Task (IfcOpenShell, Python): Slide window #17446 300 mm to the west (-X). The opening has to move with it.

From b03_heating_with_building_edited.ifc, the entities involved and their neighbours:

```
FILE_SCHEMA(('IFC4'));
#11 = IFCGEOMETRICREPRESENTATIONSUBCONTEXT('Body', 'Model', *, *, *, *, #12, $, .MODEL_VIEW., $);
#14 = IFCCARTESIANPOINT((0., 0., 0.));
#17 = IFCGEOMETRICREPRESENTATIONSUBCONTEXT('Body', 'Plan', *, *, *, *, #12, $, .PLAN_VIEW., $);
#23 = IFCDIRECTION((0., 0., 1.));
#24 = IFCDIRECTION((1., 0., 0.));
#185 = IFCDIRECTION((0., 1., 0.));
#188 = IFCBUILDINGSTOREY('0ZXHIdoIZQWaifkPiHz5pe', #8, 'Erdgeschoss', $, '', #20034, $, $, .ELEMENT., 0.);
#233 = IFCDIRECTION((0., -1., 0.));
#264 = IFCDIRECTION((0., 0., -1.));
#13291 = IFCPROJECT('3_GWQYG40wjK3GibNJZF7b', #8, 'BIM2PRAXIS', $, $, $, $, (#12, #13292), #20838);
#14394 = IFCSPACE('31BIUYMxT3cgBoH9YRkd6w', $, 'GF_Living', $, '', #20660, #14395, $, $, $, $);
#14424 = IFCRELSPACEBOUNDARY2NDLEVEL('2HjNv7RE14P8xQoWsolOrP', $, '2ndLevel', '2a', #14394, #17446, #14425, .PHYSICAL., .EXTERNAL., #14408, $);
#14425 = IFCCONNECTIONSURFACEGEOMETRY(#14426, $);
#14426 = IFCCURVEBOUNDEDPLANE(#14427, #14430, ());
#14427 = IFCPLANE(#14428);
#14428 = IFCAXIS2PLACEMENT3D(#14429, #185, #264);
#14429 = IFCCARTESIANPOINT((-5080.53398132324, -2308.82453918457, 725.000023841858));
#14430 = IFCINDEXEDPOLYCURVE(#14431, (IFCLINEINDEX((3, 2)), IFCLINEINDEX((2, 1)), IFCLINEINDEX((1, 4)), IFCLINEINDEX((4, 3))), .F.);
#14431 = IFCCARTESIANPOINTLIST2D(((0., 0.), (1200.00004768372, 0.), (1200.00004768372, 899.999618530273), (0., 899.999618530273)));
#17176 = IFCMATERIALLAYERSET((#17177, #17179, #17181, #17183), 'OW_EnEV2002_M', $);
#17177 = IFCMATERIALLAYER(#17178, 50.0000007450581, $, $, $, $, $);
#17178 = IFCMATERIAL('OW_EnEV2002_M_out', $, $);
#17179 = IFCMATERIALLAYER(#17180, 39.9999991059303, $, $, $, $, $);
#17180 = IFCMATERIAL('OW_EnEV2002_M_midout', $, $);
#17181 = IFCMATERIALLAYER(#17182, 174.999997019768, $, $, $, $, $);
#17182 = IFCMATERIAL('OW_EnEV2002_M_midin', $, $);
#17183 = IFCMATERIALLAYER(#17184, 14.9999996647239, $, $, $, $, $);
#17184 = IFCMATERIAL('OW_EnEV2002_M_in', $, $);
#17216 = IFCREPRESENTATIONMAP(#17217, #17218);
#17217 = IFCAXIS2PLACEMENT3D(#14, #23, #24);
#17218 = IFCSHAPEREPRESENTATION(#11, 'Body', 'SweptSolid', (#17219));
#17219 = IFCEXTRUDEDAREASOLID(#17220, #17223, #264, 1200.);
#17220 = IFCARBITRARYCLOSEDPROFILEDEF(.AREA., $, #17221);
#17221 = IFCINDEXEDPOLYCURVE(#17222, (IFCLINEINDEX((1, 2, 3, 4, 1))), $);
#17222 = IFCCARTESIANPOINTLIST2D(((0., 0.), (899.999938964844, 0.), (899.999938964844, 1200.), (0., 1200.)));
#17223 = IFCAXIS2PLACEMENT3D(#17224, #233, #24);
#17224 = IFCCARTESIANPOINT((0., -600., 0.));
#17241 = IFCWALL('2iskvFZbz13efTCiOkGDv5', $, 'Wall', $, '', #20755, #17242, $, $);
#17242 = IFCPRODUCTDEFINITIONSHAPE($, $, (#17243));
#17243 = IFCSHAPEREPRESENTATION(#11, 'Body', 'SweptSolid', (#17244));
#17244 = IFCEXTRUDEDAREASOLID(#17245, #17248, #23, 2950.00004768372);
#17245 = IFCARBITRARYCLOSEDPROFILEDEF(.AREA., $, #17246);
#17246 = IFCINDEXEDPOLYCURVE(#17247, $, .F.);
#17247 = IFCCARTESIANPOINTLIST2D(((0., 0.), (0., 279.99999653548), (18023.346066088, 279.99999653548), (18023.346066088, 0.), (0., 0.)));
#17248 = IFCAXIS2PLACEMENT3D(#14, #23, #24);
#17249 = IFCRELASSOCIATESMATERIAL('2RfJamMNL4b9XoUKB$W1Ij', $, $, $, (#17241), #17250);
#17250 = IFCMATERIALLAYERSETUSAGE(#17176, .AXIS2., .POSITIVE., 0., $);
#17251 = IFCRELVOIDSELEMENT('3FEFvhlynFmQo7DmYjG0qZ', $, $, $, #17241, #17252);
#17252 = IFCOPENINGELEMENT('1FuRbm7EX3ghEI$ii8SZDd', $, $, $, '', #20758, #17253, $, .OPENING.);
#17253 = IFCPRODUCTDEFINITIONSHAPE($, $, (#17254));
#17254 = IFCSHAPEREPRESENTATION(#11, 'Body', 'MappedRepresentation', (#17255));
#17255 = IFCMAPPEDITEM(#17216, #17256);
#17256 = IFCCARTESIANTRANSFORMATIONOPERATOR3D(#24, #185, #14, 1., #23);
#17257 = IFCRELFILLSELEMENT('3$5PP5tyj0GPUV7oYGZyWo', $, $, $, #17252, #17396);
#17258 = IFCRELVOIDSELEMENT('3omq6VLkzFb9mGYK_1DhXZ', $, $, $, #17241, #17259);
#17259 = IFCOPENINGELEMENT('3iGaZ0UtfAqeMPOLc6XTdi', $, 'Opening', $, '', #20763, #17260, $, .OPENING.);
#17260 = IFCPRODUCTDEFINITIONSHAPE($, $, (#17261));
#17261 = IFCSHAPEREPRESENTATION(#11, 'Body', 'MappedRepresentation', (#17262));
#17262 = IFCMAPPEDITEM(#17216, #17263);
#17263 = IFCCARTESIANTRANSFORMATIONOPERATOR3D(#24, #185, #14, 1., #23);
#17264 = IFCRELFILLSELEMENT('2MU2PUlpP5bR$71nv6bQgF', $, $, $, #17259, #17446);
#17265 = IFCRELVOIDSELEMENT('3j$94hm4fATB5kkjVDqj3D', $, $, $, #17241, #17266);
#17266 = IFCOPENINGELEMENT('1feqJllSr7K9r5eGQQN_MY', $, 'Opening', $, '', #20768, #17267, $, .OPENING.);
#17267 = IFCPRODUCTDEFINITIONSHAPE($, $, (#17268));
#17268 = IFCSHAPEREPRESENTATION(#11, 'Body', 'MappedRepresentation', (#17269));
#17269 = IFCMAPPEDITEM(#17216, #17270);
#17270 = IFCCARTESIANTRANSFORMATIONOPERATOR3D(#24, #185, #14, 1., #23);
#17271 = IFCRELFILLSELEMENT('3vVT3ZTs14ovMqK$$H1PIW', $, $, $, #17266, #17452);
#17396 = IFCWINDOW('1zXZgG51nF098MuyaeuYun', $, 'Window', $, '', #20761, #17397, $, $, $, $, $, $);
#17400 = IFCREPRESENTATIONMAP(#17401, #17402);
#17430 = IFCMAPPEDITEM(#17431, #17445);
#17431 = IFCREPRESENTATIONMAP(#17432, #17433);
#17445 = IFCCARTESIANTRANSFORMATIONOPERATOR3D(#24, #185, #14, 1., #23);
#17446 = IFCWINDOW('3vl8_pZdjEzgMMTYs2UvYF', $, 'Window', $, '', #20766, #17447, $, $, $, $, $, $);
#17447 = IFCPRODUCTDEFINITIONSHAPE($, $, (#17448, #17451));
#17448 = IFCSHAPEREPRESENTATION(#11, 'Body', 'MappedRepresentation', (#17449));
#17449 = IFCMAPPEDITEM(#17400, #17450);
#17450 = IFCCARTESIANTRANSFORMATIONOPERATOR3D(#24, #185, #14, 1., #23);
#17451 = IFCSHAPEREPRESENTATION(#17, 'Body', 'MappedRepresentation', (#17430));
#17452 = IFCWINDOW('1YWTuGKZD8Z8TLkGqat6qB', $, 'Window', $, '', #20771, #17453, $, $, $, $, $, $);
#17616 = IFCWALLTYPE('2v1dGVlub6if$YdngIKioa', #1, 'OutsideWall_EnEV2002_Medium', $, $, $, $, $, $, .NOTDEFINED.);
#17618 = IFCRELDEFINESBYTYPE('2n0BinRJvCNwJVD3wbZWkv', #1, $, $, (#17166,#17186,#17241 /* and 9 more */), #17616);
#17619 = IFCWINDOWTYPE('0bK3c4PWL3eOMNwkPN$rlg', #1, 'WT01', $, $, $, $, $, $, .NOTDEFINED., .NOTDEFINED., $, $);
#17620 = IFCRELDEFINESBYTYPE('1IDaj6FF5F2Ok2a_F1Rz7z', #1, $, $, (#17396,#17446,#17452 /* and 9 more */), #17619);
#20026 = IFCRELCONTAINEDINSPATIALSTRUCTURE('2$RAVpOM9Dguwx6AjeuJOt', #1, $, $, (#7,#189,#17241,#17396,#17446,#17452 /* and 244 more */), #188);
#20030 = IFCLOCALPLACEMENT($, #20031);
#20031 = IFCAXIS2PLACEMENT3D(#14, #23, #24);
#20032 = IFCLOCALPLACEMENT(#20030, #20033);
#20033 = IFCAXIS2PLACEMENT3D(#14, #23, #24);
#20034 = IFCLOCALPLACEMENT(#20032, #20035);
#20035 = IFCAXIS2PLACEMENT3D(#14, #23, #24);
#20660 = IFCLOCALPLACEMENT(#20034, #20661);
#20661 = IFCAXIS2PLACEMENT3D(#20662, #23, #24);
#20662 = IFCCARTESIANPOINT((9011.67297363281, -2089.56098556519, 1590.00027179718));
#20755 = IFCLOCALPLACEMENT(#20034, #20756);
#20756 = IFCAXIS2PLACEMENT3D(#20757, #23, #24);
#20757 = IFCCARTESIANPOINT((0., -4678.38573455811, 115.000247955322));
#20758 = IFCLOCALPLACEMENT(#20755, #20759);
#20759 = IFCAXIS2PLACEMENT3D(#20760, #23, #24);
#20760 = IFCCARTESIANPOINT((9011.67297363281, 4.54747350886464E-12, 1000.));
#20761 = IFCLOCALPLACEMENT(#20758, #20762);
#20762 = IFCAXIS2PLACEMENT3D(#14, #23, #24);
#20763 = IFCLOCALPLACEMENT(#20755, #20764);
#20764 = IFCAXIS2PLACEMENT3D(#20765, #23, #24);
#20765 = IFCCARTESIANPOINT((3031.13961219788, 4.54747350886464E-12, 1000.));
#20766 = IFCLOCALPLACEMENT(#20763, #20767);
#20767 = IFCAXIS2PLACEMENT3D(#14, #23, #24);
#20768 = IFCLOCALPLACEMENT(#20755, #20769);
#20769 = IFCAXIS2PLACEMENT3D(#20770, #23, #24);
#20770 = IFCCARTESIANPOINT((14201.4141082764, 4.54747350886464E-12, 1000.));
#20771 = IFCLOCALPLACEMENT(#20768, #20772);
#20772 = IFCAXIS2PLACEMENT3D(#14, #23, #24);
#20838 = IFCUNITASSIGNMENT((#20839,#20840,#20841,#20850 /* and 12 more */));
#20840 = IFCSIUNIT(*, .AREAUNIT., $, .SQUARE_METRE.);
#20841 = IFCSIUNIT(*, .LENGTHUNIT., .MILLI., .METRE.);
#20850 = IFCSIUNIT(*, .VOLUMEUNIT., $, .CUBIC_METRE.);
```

```python
import numpy as np
import ifcopenshell
import ifcopenshell.api.geometry
import ifcopenshell.util.placement

model = ifcopenshell.open("b03_heating_with_building_edited.ifc")

window = model.by_guid("3vl8_pZdjEzgMMTYs2UvYF")
opening = window.FillsVoids[0].RelatingOpeningElement
wall = opening.VoidsElements[0].RelatingBuildingElement

wall_matrix = ifcopenshell.util.placement.get_local_placement(wall.ObjectPlacement)
shift = wall_matrix[:3, 0] * -300.0
before = ifcopenshell.util.placement.get_local_placement(window.ObjectPlacement)[:3, 3].copy()

# The window is placed relative to its opening, so it follows when the opening moves.
matrix = ifcopenshell.util.placement.get_local_placement(opening.ObjectPlacement)
matrix[:3, 3] += shift
ifcopenshell.api.geometry.edit_object_placement(
    model, product=opening, matrix=matrix, is_si=False, should_transform_children=True
)

# Space boundary surfaces are stored in each space's coordinates; move them too.
for rel in window.ProvidesBoundaries:
    if not rel.ConnectionGeometry:
        continue
    surface = rel.ConnectionGeometry.SurfaceOnRelatingElement.BasisSurface
    space_matrix = ifcopenshell.util.placement.get_local_placement(rel.RelatingSpace.ObjectPlacement)
    point = np.array(surface.Position.Location.Coordinates) + space_matrix[:3, :3].T @ shift
    surface.Position = model.createIfcAxis2Placement3D(
        model.createIfcCartesianPoint(point.tolist()), surface.Position.Axis, surface.Position.RefDirection
    )

after = ifcopenshell.util.placement.get_local_placement(window.ObjectPlacement)[:3, 3]
print("window moved by", (after - before).round(3) + 0.0)

model.write("b03_heating_with_building_edited-out.ifc")
```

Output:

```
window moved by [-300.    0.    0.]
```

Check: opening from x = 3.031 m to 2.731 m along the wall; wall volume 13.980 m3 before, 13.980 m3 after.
